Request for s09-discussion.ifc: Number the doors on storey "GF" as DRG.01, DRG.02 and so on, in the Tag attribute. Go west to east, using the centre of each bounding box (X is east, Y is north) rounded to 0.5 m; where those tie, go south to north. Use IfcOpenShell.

First a look at what the model holds.

```python
import ifcopenshell
import ifcopenshell.util.element
import ifcopenshell.util.placement

model = ifcopenshell.open("s09-discussion.ifc")
print(model.schema)
storey = next(s for s in model.by_type("IfcBuildingStorey") if s.Name == "GF")
doors = [e for e in ifcopenshell.util.element.get_decomposition(storey) if e.is_a("IfcDoor")]
for e in sorted(doors, key=lambda e: e.id()):
    origin = ifcopenshell.util.placement.get_local_placement(e.ObjectPlacement)[:3, 3]
    print(e.id(), e.Tag, e.Name, origin.round(2) + 0.0, sep=" | ")
```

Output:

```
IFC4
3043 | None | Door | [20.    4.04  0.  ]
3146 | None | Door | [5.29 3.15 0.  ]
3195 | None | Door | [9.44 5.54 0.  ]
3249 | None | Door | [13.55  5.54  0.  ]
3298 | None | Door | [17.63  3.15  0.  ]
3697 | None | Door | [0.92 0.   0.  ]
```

```python
import ifcopenshell
import ifcopenshell.geom
import ifcopenshell.util.element
import ifcopenshell.util.shape

model = ifcopenshell.open("s09-discussion.ifc")
settings = ifcopenshell.geom.settings()
settings.set("use-world-coords", True)


def centre(element):
    shape = ifcopenshell.geom.create_shape(settings, element)
    return ifcopenshell.util.shape.get_bbox_centroid(shape.geometry)


storey = next(s for s in model.by_type("IfcBuildingStorey") if s.Name == "GF")
doors = [e for e in ifcopenshell.util.element.get_decomposition(storey) if e.is_a("IfcDoor")]

# Insertion points can sit at a corner or the storey origin, so sort by the geometry (in metres).
centres = {e: centre(e) for e in doors}
doors.sort(key=lambda e: (round(centres[e][0] / 0.5), centres[e][1]))

for i, e in enumerate(doors, start=1):
    number = f"DRG.{i:02d}"
    e.Tag = number
    print(e.id(), number)

model.write("s09-discussion_edited.ifc")
```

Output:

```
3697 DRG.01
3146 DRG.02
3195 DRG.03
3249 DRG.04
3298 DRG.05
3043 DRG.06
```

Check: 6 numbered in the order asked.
